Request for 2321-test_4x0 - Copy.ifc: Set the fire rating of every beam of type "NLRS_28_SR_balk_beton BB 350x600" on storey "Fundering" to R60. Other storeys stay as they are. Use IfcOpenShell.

First a look at what the model holds.

```python
import ifcopenshell
import ifcopenshell.util.element

model = ifcopenshell.open("2321-test_4x0 - Copy.ifc")
print(model.schema)
storey = next(s for s in model.by_type("IfcBuildingStorey") if s.Name == "Fundering")
beams = [e for e in ifcopenshell.util.element.get_decomposition(storey) if e.is_a("IfcBeam")]
seen = {}
for e in beams:
    element_type = ifcopenshell.util.element.get_type(e)
    key = (element_type.Name if element_type != e and element_type else None, ifcopenshell.util.element.get_pset(e, "Pset_BeamCommon", "FireRating"))
    seen[key] = seen.get(key, 0) + 1
for (name, value), count in sorted(seen.items(), key=str):
    print(count, "x", name, "|", value)
```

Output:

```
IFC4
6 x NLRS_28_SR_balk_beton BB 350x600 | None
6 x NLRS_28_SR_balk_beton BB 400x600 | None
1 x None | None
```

```python
import ifcopenshell
import ifcopenshell.api.pset
import ifcopenshell.util.element

model = ifcopenshell.open("2321-test_4x0 - Copy.ifc")

storey = next(s for s in model.by_type("IfcBuildingStorey") if s.Name == "Fundering")
beams = [e for e in ifcopenshell.util.element.get_decomposition(storey) if e.is_a("IfcBeam")]

count = 0
for e in beams:
    element_type = ifcopenshell.util.element.get_type(e)
    if element_type in (None, e) or element_type.Name != "NLRS_28_SR_balk_beton BB 350x600":
        continue
    # add_pset returns the element's existing set when there is one.
    pset = ifcopenshell.api.pset.add_pset(model, product=e, name="Pset_BeamCommon")
    ifcopenshell.api.pset.edit_pset(model, pset=pset, properties={"FireRating": "R60"})
    count += 1

print(count, "beams updated")

model.write("2321-test_4x0 - Copy-out.ifc")
```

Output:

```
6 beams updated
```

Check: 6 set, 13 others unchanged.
